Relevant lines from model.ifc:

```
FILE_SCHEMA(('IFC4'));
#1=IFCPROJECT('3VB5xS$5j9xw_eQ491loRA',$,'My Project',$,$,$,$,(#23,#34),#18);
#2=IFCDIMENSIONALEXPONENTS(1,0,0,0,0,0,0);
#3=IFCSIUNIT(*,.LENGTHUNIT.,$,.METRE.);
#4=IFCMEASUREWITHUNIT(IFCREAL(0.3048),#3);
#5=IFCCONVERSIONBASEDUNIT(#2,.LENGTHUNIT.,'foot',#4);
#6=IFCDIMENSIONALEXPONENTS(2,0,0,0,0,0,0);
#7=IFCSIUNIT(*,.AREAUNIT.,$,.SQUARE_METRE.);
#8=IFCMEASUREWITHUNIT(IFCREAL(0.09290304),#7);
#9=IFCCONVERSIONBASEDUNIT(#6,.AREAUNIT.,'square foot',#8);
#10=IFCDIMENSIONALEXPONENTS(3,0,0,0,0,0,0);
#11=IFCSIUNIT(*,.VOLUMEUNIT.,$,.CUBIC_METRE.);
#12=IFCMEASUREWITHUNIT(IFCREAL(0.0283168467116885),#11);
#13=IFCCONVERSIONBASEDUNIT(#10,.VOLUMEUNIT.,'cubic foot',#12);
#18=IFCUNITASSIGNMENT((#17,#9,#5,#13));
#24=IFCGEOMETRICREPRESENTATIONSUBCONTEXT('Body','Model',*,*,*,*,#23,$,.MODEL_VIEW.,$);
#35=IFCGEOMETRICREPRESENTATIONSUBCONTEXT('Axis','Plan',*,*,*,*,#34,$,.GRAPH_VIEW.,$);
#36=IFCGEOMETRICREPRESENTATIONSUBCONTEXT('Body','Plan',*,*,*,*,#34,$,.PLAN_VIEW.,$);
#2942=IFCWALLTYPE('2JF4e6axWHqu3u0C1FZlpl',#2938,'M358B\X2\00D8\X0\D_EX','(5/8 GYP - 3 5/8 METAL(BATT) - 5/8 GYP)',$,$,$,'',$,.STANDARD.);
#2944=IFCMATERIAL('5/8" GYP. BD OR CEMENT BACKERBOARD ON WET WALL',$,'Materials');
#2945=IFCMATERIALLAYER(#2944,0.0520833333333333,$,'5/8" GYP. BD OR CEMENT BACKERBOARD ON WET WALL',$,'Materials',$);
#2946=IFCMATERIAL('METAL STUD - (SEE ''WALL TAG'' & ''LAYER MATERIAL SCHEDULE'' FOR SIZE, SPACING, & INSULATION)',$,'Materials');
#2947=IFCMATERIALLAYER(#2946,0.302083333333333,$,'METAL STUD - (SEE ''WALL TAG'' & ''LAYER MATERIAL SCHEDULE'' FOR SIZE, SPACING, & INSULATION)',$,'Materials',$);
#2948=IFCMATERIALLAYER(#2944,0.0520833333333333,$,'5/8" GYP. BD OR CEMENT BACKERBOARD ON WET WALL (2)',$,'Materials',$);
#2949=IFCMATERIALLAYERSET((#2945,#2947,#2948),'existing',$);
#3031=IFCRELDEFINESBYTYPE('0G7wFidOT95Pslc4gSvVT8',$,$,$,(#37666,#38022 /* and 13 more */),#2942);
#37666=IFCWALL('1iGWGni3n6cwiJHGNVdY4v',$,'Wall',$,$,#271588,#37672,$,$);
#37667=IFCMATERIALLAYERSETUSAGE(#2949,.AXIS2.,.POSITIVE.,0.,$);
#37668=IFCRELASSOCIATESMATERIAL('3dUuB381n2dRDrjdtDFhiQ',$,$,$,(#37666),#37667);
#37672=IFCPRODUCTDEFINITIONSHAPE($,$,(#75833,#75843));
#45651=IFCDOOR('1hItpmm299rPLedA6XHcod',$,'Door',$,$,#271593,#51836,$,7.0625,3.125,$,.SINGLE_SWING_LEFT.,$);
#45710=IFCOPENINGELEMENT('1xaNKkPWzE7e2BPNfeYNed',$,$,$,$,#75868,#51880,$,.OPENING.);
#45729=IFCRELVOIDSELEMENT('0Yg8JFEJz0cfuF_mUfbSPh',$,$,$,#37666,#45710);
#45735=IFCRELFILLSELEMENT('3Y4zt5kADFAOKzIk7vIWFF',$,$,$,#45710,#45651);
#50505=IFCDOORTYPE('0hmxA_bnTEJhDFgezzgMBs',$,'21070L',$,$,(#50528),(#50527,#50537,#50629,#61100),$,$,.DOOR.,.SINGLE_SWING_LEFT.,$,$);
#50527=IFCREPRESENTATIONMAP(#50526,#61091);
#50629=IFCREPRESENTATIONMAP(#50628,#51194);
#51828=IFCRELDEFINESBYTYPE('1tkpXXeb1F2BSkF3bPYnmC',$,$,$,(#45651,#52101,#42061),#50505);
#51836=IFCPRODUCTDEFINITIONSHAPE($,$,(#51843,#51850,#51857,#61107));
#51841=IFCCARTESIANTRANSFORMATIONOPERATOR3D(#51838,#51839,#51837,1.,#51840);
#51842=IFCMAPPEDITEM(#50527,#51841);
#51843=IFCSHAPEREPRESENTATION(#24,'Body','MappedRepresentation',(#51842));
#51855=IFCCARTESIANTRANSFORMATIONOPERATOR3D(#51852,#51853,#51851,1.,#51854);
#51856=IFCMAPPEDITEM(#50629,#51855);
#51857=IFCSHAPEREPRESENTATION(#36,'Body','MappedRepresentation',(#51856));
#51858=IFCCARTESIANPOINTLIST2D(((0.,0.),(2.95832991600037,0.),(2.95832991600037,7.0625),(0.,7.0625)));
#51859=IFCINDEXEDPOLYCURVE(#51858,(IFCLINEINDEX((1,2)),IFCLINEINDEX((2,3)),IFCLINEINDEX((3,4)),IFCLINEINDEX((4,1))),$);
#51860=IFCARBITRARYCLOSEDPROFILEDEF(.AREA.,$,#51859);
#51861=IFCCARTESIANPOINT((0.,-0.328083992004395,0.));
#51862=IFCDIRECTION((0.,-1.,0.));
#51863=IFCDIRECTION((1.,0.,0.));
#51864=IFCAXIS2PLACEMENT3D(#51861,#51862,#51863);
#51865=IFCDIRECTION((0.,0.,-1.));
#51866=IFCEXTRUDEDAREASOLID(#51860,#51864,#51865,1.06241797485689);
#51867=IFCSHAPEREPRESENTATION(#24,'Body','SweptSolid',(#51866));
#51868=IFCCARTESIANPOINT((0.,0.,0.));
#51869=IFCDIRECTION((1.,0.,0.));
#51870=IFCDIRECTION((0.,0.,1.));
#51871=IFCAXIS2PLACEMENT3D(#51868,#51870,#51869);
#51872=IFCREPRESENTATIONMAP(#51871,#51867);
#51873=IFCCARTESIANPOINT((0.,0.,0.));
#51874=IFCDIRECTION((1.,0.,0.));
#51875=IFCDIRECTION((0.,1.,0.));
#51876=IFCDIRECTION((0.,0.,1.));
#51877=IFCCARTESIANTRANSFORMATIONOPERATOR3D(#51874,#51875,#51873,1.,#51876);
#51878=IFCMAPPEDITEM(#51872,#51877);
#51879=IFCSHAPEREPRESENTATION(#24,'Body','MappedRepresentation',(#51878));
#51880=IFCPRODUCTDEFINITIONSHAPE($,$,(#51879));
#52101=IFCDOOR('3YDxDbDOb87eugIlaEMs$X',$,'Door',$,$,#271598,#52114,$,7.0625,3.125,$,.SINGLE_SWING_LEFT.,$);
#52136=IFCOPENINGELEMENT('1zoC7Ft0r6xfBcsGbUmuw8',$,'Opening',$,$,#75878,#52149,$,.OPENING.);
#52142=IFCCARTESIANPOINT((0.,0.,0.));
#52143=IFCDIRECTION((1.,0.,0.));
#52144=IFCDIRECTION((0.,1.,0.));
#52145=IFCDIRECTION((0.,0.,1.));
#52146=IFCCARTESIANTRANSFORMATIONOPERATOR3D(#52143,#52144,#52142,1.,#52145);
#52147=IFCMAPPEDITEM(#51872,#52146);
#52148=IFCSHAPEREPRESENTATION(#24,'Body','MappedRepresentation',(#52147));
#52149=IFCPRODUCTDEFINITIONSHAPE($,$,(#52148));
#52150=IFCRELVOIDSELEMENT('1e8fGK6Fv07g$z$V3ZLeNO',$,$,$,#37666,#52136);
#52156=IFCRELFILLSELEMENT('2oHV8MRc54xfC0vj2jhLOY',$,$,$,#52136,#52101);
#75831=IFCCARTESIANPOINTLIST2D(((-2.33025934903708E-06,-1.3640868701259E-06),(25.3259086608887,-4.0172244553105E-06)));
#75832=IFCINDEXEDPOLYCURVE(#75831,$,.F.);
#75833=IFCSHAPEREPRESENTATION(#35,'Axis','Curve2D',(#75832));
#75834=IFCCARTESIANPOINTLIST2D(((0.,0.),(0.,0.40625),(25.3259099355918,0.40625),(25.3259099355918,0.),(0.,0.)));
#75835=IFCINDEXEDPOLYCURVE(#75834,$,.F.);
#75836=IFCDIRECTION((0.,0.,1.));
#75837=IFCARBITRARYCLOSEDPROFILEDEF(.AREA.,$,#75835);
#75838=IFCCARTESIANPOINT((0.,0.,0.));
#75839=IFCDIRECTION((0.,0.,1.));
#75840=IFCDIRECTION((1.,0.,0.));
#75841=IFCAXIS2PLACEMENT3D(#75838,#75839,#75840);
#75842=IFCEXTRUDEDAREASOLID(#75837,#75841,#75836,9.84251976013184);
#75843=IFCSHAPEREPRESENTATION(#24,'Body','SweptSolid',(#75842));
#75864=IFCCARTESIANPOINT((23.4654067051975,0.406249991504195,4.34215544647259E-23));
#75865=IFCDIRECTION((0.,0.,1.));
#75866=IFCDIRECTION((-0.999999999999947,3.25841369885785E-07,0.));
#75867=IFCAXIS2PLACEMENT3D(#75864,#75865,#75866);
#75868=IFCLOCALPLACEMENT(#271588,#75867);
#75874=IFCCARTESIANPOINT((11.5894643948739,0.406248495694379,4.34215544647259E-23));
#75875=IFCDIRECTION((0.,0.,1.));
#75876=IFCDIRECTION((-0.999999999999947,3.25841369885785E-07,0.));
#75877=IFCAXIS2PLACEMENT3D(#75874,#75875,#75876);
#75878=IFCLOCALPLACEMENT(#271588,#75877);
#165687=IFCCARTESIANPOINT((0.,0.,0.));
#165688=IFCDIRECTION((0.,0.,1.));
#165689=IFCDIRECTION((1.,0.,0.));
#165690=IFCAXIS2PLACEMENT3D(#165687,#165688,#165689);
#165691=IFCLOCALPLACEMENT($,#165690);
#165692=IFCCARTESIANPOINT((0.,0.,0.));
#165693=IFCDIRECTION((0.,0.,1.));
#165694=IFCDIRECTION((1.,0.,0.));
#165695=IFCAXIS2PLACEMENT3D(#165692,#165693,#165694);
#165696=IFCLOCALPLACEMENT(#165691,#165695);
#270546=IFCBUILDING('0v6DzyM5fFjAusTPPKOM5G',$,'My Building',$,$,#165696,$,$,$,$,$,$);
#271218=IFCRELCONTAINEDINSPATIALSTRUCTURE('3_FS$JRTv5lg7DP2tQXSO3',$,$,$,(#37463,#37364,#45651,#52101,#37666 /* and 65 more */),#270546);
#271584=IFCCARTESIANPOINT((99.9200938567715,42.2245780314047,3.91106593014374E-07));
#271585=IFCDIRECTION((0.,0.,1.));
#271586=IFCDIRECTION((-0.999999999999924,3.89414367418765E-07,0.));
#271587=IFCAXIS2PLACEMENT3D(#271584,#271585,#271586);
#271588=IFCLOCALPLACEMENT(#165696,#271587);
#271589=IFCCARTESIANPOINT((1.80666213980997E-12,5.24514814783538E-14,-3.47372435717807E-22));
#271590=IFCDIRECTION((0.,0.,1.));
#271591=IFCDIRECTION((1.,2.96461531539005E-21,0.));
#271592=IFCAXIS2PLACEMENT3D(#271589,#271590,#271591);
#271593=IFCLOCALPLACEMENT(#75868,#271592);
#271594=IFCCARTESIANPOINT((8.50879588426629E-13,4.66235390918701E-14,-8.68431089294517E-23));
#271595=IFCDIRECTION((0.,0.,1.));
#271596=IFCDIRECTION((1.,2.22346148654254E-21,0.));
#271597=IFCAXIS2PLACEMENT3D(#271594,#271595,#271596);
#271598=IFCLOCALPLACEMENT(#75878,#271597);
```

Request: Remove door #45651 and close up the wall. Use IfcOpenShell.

```python
import ifcopenshell
import ifcopenshell.api.feature
import ifcopenshell.api.root
import ifcopenshell.geom
import ifcopenshell.util.shape

model = ifcopenshell.open("model.ifc")
settings = ifcopenshell.geom.settings()


def volume(element):
    """Net volume in cubic metres, openings subtracted."""
    shape = ifcopenshell.geom.create_shape(settings, element)
    return ifcopenshell.util.shape.get_volume(shape.geometry)


door = model.by_guid("1hItpmm299rPLedA6XHcod")
opening = door.FillsVoids[0].RelatingOpeningElement
wall = opening.VoidsElements[0].RelatingBuildingElement
before = volume(wall)

ifcopenshell.api.root.remove_product(model, product=door)
ifcopenshell.api.feature.remove_feature(model, feature=opening)

after = volume(wall)

print(f"wall volume {before:.3f} -> {after:.3f} m3")

model.write("model_updated.ifc")
```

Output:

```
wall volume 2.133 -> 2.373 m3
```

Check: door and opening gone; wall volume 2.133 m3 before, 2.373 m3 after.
